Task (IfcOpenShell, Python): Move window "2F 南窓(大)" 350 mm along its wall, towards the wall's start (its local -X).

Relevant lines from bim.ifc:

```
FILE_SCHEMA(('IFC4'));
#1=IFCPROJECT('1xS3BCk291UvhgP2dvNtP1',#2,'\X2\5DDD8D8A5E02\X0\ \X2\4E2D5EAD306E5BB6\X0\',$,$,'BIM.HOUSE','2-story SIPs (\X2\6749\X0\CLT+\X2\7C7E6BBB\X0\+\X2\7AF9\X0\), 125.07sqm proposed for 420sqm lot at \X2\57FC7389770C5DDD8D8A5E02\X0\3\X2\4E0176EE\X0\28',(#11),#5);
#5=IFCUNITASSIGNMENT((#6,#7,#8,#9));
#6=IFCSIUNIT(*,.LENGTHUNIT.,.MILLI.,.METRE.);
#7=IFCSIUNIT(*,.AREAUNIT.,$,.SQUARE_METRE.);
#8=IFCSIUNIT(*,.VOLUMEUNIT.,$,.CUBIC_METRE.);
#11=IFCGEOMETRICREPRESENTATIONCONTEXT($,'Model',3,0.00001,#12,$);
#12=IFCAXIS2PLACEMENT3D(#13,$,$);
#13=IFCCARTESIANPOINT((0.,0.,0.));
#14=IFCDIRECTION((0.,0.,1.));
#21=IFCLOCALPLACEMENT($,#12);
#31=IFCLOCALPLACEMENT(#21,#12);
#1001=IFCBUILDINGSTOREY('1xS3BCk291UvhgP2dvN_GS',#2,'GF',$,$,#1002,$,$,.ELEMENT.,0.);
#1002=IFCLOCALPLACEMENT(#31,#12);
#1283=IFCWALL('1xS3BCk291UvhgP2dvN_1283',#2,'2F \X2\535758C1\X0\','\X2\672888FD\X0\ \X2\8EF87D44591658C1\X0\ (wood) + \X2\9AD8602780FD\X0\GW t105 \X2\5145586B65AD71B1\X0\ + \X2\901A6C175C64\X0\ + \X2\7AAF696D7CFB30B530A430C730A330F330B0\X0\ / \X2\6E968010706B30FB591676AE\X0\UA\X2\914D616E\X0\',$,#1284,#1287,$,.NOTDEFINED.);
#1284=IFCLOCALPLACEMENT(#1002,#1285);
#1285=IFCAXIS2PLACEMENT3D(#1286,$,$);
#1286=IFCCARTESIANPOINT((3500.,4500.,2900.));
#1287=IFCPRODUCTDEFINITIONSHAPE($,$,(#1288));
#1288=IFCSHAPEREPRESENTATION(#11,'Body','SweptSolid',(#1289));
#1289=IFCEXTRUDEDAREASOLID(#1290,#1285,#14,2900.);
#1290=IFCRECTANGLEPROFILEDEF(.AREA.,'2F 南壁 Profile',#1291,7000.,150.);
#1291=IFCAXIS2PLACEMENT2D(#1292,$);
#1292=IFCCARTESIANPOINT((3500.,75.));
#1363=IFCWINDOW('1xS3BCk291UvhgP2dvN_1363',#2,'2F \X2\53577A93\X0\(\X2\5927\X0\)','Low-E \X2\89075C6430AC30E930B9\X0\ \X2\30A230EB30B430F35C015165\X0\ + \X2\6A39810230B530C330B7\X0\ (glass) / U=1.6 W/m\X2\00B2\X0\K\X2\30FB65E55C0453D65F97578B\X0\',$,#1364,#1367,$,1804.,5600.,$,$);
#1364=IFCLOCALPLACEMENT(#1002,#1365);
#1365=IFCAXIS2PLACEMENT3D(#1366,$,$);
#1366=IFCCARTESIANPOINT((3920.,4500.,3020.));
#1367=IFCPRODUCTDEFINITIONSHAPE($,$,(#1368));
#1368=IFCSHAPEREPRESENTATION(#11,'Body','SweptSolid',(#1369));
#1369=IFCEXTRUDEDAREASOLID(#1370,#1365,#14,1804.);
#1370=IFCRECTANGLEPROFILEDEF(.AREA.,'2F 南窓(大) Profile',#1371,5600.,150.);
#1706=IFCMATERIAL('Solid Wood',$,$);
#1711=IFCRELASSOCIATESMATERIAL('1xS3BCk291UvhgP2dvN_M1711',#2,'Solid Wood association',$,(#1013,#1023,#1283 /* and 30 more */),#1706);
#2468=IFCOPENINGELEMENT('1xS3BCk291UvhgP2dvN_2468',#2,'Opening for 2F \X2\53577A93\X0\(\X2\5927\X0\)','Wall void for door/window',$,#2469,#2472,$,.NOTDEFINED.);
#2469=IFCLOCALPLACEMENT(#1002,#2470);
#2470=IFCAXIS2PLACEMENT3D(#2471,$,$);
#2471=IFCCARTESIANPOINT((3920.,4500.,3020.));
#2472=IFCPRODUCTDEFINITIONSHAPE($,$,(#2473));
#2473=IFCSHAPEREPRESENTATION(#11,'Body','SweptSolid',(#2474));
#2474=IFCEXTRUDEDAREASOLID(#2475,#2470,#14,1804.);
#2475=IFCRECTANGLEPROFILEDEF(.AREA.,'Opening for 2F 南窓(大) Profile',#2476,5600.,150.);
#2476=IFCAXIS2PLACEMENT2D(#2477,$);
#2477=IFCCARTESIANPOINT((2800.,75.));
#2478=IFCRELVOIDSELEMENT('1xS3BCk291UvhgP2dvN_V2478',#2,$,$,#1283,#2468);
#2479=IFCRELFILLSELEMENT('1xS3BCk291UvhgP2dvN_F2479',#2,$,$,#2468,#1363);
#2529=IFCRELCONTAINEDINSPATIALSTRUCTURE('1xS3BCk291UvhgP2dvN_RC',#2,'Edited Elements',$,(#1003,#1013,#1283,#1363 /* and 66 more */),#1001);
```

```python
import ifcopenshell
import ifcopenshell.api.geometry
import ifcopenshell.util.placement
import ifcopenshell.util.unit

model = ifcopenshell.open("bim.ifc")
unit_scale = ifcopenshell.util.unit.calculate_unit_scale(model)

window = model.by_guid("1xS3BCk291UvhgP2dvN_1363")
opening = window.FillsVoids[0].RelatingOpeningElement
wall = opening.VoidsElements[0].RelatingBuildingElement

wall_matrix = ifcopenshell.util.placement.get_local_placement(wall.ObjectPlacement)
shift = wall_matrix[:3, 0] * -0.35 / unit_scale
before = ifcopenshell.util.placement.get_local_placement(window.ObjectPlacement)[:3, 3].copy()

# The window is not placed relative to its opening, so move both.
for product in (opening, window):
    matrix = ifcopenshell.util.placement.get_local_placement(product.ObjectPlacement)
    matrix[:3, 3] += shift
    ifcopenshell.api.geometry.edit_object_placement(model, product=product, matrix=matrix, is_si=False)

after = ifcopenshell.util.placement.get_local_placement(window.ObjectPlacement)[:3, 3]
print("window moved by", (after - before).round(3) + 0.0)

model.write("bim_v2.ifc")
```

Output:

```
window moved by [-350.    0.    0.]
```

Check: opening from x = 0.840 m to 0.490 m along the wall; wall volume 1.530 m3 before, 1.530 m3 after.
